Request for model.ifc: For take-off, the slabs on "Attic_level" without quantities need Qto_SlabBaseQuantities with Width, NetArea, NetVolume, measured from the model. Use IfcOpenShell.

First a look at what the model holds.

```python
import ifcopenshell
import ifcopenshell.util.element
import ifcopenshell.util.unit

model = ifcopenshell.open("model.ifc")
print(model.schema)
for unit_type in ("LENGTHUNIT", "AREAUNIT", "VOLUMEUNIT"):
    print(unit_type, ifcopenshell.util.unit.calculate_unit_scale(model, unit_type))
storey = next(s for s in model.by_type("IfcBuildingStorey") if s.Name == "Attic_level")
slabs = [e for e in ifcopenshell.util.element.get_decomposition(storey) if e.is_a("IfcSlab")]
for e in sorted(slabs, key=lambda e: e.id()):
    print(e.id(), e.is_a(), e.Name, list(ifcopenshell.util.element.get_psets(e, qtos_only=True)), sep=" | ")
```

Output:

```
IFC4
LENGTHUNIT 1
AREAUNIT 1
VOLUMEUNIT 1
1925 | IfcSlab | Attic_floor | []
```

```python
import ifcopenshell
import ifcopenshell.api.pset
import ifcopenshell.geom
import ifcopenshell.util.element
import ifcopenshell.util.shape
import ifcopenshell.util.unit

model = ifcopenshell.open("model.ifc")
unit_scale = ifcopenshell.util.unit.calculate_unit_scale(model)
area_scale = ifcopenshell.util.unit.calculate_unit_scale(model, "AREAUNIT")
volume_scale = ifcopenshell.util.unit.calculate_unit_scale(model, "VOLUMEUNIT")
settings = ifcopenshell.geom.settings()

storey = next(s for s in model.by_type("IfcBuildingStorey") if s.Name == "Attic_level")
slabs = [e for e in ifcopenshell.util.element.get_decomposition(storey) if e.is_a("IfcSlab")]

for e in sorted(slabs, key=lambda e: e.id()):
    if ifcopenshell.util.element.get_psets(e, qtos_only=True, should_inherit=False):
        continue
    # Geometry comes back in metres, in the element's own axes.
    shape = ifcopenshell.geom.create_shape(settings, e)
    values = {
        "Width": ifcopenshell.util.shape.get_z(shape.geometry) / unit_scale,
        "NetArea": ifcopenshell.util.shape.get_footprint_area(shape.geometry) / area_scale,
        "NetVolume": ifcopenshell.util.shape.get_volume(shape.geometry) / volume_scale,
    }
    qto = ifcopenshell.api.pset.add_qto(model, product=e, name="Qto_SlabBaseQuantities")
    ifcopenshell.api.pset.edit_qto(model, qto=qto, properties=values)
    print(e.id(), {k: round(v, 3) for k, v in values.items()})

model.write("model_v2.ifc")
```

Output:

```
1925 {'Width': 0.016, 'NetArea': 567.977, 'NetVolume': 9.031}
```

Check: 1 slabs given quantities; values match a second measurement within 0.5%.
